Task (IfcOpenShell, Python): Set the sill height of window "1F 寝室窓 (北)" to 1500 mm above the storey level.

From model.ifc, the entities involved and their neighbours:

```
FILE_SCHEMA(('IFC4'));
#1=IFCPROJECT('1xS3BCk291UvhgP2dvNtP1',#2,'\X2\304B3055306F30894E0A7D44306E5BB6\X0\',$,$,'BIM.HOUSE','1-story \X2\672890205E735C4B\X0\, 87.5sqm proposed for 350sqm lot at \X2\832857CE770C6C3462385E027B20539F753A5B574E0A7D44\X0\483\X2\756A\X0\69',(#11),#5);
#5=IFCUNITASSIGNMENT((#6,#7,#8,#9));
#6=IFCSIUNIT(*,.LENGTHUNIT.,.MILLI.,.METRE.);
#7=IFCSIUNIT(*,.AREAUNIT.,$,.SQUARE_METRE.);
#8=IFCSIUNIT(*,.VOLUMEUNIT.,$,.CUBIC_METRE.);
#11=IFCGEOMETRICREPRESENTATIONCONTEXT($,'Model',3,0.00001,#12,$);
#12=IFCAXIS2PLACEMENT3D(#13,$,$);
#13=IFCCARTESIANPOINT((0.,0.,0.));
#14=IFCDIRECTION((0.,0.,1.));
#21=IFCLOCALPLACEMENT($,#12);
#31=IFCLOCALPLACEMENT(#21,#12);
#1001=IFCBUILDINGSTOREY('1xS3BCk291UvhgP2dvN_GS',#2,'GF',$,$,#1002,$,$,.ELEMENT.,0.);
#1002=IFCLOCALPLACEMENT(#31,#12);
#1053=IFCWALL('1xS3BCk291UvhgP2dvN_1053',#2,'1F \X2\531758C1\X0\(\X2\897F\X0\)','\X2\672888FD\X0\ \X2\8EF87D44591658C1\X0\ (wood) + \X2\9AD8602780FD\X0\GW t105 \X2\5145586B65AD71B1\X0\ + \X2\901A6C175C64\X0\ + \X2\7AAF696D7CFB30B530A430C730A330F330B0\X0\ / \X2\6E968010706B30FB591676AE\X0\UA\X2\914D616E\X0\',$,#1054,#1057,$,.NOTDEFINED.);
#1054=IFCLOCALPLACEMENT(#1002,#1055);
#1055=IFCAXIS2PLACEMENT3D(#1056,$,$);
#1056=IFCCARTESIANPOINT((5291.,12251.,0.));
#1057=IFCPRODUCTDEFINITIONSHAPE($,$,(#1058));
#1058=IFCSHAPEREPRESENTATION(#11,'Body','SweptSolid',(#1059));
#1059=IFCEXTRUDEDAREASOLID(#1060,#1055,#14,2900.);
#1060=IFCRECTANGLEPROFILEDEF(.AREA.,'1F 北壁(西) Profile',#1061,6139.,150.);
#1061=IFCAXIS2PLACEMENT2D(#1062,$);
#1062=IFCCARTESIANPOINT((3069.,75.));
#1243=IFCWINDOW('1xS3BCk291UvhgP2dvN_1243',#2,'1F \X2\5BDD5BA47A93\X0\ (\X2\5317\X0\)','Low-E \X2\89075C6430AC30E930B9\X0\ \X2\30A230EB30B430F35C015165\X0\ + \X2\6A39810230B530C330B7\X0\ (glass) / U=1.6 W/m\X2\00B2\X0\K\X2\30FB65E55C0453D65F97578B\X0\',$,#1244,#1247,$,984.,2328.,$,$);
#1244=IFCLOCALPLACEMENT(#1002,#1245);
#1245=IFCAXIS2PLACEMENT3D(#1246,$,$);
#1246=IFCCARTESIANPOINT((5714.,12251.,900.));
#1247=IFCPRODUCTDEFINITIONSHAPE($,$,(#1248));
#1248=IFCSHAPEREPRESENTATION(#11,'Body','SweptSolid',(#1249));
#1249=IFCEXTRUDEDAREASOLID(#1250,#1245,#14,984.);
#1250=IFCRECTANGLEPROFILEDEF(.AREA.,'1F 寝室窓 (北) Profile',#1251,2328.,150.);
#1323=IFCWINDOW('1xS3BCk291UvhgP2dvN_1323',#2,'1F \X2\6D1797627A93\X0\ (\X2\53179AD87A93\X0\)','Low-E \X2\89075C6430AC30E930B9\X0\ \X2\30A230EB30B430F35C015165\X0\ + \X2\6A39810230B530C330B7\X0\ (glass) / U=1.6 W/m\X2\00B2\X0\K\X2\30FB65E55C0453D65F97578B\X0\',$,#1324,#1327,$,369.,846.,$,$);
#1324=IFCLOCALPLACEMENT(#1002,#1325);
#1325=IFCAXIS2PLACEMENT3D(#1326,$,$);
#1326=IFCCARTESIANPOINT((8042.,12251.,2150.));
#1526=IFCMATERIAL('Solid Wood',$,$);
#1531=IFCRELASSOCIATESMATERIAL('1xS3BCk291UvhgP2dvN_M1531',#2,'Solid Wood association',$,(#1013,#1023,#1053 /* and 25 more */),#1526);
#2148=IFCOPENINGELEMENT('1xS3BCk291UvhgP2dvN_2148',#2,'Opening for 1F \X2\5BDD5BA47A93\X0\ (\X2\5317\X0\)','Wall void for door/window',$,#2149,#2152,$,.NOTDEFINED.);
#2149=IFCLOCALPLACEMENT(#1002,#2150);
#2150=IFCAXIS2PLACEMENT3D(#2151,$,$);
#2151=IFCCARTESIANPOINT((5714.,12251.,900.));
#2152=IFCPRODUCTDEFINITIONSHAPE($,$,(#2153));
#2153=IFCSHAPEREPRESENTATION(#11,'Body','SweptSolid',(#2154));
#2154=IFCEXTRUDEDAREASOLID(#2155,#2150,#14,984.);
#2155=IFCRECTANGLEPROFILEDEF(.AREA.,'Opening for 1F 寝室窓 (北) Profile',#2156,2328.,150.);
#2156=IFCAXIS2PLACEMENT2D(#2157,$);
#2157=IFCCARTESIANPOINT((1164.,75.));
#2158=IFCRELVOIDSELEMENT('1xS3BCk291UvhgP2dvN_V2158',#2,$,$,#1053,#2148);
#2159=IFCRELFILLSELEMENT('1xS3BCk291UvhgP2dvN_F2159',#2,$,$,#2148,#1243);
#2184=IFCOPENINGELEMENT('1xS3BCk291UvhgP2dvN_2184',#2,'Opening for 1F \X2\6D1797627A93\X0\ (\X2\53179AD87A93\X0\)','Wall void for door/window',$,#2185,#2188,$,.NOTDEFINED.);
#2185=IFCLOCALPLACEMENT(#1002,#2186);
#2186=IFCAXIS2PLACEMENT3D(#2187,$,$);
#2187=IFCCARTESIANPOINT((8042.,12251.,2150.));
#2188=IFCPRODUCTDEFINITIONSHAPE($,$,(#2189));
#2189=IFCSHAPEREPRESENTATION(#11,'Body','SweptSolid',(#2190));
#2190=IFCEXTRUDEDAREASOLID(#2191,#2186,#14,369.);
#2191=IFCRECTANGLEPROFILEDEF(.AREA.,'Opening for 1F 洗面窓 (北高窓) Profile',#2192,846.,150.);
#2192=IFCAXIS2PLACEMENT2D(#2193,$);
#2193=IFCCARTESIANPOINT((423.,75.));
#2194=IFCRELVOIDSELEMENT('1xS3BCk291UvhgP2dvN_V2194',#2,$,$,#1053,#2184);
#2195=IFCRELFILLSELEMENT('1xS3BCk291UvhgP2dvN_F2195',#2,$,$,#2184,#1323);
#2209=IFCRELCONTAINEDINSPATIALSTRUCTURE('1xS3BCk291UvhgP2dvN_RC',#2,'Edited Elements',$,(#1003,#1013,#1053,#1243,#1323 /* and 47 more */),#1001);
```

```python
import numpy as np
import ifcopenshell
import ifcopenshell.api.geometry
import ifcopenshell.geom
import ifcopenshell.util.element
import ifcopenshell.util.placement
import ifcopenshell.util.shape
import ifcopenshell.util.unit

model = ifcopenshell.open("model.ifc")
unit_scale = ifcopenshell.util.unit.calculate_unit_scale(model)

window = model.by_id(1243)
opening = window.FillsVoids[0].RelatingOpeningElement
storey = ifcopenshell.util.element.get_container(window, ifc_class="IfcBuildingStorey")
level = ifcopenshell.util.placement.get_local_placement(storey.ObjectPlacement)[2, 3]

# The opening's origin need not be at the sill, so measure its lowest point.
shape = ifcopenshell.geom.create_shape(ifcopenshell.geom.settings(), opening)
bottom = ifcopenshell.util.shape.get_shape_bottom_elevation(shape, shape.geometry) / unit_scale
dz = level + 1.5 / unit_scale - bottom

shift = np.array([0.0, 0.0, dz])
# The window is not placed relative to its opening, so move both.
for product in (opening, window):
    matrix = ifcopenshell.util.placement.get_local_placement(product.ObjectPlacement)
    matrix[:3, 3] += shift
    ifcopenshell.api.geometry.edit_object_placement(model, product=product, matrix=matrix, is_si=False)

print(f"moved by {dz * unit_scale:+.3f} m")

model.write("model_updated.ifc")
```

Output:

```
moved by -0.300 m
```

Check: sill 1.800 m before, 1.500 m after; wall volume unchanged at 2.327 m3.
